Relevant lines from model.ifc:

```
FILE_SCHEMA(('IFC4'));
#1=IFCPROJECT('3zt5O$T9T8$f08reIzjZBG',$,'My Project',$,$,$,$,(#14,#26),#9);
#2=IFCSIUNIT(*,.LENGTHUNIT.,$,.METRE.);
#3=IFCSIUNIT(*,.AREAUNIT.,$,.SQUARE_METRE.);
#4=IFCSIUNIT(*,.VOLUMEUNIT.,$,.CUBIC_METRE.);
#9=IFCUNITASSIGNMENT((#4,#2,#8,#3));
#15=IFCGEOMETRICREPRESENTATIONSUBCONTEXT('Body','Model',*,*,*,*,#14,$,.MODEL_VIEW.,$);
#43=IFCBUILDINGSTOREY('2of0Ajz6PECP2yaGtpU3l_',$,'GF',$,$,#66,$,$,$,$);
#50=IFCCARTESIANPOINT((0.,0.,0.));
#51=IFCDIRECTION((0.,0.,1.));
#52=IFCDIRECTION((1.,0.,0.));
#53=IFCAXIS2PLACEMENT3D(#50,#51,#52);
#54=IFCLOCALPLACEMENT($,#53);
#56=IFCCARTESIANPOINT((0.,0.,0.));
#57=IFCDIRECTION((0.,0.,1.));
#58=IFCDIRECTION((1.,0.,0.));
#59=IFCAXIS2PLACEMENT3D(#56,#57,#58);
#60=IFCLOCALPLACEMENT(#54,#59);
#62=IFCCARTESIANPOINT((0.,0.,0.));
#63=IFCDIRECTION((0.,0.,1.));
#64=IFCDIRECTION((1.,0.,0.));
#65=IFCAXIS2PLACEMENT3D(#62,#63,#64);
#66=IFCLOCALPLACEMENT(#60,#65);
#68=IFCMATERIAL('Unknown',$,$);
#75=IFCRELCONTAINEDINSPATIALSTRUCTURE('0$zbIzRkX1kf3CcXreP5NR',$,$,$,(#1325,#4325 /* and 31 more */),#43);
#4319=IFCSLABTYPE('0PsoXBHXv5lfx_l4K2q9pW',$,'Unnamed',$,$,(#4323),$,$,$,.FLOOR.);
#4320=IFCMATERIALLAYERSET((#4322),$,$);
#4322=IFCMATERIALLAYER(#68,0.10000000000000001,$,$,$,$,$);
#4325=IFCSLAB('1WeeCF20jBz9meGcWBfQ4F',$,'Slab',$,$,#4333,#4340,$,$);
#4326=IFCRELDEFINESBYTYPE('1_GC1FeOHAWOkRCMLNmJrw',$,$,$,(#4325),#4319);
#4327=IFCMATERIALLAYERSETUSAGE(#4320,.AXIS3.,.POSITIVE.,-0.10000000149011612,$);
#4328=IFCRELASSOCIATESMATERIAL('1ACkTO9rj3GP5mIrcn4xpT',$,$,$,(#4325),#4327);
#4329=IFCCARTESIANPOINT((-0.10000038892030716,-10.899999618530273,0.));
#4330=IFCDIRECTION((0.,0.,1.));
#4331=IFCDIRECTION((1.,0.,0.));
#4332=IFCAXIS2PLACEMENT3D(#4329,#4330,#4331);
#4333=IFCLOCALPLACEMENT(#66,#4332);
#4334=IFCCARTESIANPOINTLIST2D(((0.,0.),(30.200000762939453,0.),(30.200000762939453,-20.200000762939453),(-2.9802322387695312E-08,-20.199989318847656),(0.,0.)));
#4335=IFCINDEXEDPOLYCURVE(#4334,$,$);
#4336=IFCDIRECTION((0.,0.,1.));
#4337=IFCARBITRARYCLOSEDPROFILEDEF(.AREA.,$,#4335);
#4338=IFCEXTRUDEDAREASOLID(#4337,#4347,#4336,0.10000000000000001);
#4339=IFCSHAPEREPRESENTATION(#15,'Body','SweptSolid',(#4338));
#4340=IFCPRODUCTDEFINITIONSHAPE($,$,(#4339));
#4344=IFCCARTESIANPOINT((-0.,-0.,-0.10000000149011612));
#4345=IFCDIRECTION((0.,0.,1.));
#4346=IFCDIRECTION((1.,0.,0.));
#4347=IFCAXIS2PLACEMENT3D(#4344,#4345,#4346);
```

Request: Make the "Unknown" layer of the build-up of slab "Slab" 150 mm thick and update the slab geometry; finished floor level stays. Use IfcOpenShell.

```python
import ifcopenshell
import ifcopenshell.util.element
import ifcopenshell.util.representation

model = ifcopenshell.open("model.ifc")

layer_set = model.by_id(4320)
layer = next(l for l in layer_set.MaterialLayers if l.Material and l.Material.Name == "Unknown")
change = 0.15 - layer.LayerThickness
layer.LayerThickness += change

# Geometry does not follow the layer set by itself.
slabs = [e for e in ifcopenshell.util.element.get_elements_by_material(model, layer_set) if e.is_a("IfcSlab")]
for slab in sorted(slabs, key=lambda e: e.id()):
    body = ifcopenshell.util.representation.get_representation(slab, "Model", "Body")
    solid = body.Items[0]
    old_depth = solid.Depth
    solid.Depth += change
    # Extruded upwards: lower the start of the extrusion so the top stays.
    x, y, z = solid.Position.Location.Coordinates
    solid.Position.Location = model.createIfcCartesianPoint((x, y, z - change))
    print(slab.id(), f"{old_depth:g} -> {solid.Depth:g}")

# The layers are counted up from the underside, which has moved.
for usage in {ifcopenshell.util.element.get_material(slab) for slab in slabs}:
    usage.OffsetFromReferenceLine -= change

model.write("model_updated.ifc")
```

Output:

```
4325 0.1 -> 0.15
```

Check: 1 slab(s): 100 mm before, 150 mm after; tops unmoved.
